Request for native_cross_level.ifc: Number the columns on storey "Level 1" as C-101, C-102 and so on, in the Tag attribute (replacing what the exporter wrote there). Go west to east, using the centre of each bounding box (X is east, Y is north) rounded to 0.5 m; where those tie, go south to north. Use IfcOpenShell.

First a look at what the model holds.

```python
import ifcopenshell
import ifcopenshell.util.element
import ifcopenshell.util.placement

model = ifcopenshell.open("native_cross_level.ifc")
print(model.schema)
storey = next(s for s in model.by_type("IfcBuildingStorey") if s.Name == "Level 1")
columns = [e for e in ifcopenshell.util.element.get_decomposition(storey) if e.is_a("IfcColumn")]
for e in sorted(columns, key=lambda e: e.id()):
    origin = ifcopenshell.util.placement.get_local_placement(e.ObjectPlacement)[:3, 3]
    print(e.id(), e.Tag, e.Name, origin.round(2) + 0.0, sep=" | ")
```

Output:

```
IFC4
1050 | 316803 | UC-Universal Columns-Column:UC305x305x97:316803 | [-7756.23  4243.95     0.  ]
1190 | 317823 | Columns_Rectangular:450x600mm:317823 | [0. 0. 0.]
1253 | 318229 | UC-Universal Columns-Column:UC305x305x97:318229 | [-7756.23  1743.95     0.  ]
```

```python
import ifcopenshell
import ifcopenshell.geom
import ifcopenshell.util.element
import ifcopenshell.util.shape

model = ifcopenshell.open("native_cross_level.ifc")
settings = ifcopenshell.geom.settings()
settings.set("use-world-coords", True)


def centre(element):
    shape = ifcopenshell.geom.create_shape(settings, element)
    return ifcopenshell.util.shape.get_bbox_centroid(shape.geometry)


storey = next(s for s in model.by_type("IfcBuildingStorey") if s.Name == "Level 1")
columns = [e for e in ifcopenshell.util.element.get_decomposition(storey) if e.is_a("IfcColumn")]

# Insertion points can sit at a corner or the storey origin, so sort by the geometry (in metres).
centres = {e: centre(e) for e in columns}
columns.sort(key=lambda e: (round(centres[e][0] / 0.5), centres[e][1]))

for i, e in enumerate(columns, start=1):
    number = f"C-1{i:02d}"
    e.Tag = number
    print(e.id(), number)

model.write("native_cross_level_v2.ifc")
```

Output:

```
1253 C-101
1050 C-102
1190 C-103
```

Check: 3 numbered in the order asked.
